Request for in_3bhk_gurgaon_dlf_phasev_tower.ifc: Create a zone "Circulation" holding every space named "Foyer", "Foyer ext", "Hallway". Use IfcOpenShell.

First a look at what the model holds.

```python
import ifcopenshell

model = ifcopenshell.open("in_3bhk_gurgaon_dlf_phasev_tower.ifc")
print(model.schema)
seen = {}
for space in model.by_type("IfcSpace"):
    seen[space.LongName] = seen.get(space.LongName, 0) + 1
for name, count in sorted(seen.items(), key=str):
    print(count, "x", name)
print("zones:", [z.Name for z in model.by_type("IfcZone")][:20])
```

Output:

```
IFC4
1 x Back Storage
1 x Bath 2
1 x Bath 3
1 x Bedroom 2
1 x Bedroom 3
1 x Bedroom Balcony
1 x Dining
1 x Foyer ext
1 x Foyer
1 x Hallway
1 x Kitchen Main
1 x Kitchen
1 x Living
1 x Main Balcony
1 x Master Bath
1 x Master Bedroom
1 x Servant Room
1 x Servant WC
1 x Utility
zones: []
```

```python
import ifcopenshell
import ifcopenshell.api.group
import ifcopenshell.api.root

model = ifcopenshell.open("in_3bhk_gurgaon_dlf_phasev_tower.ifc")

names = {"Foyer", "Foyer ext", "Hallway"}
spaces = [s for s in model.by_type("IfcSpace") if s.LongName in names]

zone = ifcopenshell.api.root.create_entity(model, ifc_class="IfcZone", name="Circulation")
ifcopenshell.api.group.assign_group(model, products=spaces, group=zone)
print(len(spaces), "spaces in", zone.Name)

model.write("in_3bhk_gurgaon_dlf_phasev_tower_updated.ifc")
```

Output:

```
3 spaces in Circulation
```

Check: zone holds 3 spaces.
